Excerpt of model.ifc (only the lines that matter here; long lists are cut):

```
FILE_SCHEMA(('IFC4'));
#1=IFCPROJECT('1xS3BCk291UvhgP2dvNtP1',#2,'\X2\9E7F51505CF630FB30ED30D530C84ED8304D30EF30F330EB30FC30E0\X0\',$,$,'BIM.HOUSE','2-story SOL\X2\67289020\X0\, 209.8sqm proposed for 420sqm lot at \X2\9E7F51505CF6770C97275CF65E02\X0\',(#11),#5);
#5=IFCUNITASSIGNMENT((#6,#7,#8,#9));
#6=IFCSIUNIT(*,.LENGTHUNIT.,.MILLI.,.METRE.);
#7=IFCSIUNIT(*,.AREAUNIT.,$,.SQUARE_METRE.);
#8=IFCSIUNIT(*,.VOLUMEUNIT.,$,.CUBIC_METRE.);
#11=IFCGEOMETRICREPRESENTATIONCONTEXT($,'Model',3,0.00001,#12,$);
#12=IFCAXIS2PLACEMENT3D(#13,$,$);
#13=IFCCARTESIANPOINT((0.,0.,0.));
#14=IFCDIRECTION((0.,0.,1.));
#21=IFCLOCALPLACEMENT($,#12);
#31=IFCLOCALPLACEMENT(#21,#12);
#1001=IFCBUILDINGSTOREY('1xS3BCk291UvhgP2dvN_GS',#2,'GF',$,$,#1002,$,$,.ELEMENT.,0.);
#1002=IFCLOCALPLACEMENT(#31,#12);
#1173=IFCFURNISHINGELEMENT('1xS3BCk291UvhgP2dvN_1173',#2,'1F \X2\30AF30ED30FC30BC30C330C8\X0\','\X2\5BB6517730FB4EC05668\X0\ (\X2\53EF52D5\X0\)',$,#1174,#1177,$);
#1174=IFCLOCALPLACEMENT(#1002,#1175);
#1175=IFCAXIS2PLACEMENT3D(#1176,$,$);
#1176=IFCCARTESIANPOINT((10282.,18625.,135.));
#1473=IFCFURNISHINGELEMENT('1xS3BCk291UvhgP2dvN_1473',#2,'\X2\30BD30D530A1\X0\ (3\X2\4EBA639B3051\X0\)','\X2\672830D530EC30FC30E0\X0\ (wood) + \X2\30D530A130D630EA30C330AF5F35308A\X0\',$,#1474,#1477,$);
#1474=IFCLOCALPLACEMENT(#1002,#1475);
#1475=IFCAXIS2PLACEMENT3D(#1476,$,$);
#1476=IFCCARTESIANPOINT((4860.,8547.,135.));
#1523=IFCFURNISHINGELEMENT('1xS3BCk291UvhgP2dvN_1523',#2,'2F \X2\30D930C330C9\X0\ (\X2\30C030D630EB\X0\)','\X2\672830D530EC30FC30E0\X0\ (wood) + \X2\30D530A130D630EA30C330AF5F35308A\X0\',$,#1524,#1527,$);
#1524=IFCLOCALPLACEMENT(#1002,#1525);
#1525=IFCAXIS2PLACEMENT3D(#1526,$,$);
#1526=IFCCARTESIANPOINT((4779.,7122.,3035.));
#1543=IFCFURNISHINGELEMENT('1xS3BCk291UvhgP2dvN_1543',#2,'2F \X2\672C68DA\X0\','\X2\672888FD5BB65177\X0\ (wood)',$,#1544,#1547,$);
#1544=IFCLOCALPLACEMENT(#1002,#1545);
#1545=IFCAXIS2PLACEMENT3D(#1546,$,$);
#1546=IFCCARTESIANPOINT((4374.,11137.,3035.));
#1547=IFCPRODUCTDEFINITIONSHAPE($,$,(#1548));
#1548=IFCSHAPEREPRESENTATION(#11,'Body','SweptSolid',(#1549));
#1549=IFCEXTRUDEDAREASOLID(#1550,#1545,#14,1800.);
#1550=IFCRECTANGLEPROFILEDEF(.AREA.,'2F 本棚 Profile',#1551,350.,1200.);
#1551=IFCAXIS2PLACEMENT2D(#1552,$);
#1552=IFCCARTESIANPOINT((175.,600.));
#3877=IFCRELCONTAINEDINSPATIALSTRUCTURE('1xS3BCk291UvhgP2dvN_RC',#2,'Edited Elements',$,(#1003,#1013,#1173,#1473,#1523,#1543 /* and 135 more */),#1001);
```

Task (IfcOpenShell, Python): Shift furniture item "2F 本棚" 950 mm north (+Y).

```python
import ifcopenshell
import ifcopenshell.api.geometry
import ifcopenshell.util.placement
import ifcopenshell.util.unit

model = ifcopenshell.open("model.ifc")
unit_scale = ifcopenshell.util.unit.calculate_unit_scale(model)

item = model.by_id(1543)
matrix = ifcopenshell.util.placement.get_local_placement(item.ObjectPlacement)
matrix[1, 3] += 0.95 / unit_scale
ifcopenshell.api.geometry.edit_object_placement(model, product=item, matrix=matrix, is_si=False)

print(ifcopenshell.util.placement.get_local_placement(item.ObjectPlacement).round(3) + 0.0)

model.write("model_rev.ifc")
```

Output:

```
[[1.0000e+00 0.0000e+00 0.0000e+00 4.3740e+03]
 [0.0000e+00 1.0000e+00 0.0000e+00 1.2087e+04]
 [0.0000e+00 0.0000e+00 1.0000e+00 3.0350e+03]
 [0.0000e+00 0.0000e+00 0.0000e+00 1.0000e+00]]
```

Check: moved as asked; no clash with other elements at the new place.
